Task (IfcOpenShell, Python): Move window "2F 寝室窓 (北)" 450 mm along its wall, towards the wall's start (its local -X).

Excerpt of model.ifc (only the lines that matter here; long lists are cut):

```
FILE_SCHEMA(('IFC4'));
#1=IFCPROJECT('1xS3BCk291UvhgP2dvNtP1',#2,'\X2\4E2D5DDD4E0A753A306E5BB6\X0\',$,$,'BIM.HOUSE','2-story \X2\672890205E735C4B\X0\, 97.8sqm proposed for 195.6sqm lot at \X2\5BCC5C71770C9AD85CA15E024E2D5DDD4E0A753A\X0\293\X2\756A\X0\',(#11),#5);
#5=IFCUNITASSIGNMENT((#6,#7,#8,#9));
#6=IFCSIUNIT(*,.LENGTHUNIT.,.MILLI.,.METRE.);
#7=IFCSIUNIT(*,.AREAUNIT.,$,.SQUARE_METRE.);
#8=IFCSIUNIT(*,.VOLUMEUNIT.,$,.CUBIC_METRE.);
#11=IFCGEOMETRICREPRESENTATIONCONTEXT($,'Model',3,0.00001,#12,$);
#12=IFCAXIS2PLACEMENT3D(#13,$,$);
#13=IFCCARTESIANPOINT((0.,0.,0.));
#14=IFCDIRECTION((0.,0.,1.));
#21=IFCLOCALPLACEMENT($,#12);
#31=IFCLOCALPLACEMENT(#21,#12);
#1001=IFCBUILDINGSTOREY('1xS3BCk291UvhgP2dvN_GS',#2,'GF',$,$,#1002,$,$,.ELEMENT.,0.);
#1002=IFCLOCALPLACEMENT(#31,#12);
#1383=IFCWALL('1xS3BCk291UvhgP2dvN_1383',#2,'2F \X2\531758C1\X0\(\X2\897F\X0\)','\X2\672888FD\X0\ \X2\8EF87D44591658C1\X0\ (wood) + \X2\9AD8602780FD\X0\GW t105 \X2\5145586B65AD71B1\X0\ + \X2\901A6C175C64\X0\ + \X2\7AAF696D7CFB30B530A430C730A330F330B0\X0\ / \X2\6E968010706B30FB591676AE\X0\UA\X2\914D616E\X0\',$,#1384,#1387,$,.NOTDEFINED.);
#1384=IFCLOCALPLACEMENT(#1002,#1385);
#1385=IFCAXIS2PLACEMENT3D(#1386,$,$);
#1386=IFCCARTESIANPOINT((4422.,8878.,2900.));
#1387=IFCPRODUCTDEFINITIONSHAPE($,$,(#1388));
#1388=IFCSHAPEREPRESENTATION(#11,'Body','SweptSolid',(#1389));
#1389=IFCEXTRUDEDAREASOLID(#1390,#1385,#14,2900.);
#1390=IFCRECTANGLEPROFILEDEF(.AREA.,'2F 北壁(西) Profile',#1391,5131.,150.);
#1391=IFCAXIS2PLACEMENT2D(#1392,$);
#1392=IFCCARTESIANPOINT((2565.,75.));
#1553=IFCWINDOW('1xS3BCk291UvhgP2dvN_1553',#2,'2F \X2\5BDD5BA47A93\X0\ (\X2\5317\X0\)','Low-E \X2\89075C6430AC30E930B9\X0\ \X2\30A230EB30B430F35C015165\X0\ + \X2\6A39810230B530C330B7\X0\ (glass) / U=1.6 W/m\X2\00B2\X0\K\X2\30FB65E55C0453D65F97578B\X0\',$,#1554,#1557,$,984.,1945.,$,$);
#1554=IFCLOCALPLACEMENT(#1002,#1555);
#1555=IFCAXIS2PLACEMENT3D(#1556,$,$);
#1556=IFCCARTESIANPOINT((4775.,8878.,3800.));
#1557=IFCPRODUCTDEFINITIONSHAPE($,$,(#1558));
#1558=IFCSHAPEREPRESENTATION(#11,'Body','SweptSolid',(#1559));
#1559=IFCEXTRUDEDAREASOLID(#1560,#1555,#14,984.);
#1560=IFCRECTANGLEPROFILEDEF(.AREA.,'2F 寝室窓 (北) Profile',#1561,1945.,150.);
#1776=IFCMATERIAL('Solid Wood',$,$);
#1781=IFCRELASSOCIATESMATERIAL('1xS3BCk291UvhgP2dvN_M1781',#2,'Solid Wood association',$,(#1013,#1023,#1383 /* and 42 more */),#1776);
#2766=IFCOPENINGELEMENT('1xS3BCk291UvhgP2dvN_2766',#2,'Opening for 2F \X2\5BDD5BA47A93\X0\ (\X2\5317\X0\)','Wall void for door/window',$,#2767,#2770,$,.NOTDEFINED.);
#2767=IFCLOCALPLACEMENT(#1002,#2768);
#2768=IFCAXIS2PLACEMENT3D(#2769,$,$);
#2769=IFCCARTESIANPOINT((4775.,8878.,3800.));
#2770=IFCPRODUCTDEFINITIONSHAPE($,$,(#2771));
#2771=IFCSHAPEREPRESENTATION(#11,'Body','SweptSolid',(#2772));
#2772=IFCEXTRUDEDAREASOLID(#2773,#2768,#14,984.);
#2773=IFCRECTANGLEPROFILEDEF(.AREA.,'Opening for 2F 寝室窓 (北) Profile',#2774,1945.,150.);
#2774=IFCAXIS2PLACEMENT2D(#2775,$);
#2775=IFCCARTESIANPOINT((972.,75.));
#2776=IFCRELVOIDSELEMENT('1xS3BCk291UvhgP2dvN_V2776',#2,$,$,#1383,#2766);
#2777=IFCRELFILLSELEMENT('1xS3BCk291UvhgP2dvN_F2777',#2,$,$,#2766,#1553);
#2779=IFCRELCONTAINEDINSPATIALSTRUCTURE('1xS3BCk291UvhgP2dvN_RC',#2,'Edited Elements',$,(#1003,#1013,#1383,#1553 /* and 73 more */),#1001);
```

```python
import ifcopenshell
import ifcopenshell.api.geometry
import ifcopenshell.util.placement
import ifcopenshell.util.unit

model = ifcopenshell.open("model.ifc")
unit_scale = ifcopenshell.util.unit.calculate_unit_scale(model)

window = model.by_id(1553)
opening = window.FillsVoids[0].RelatingOpeningElement
wall = opening.VoidsElements[0].RelatingBuildingElement

wall_matrix = ifcopenshell.util.placement.get_local_placement(wall.ObjectPlacement)
shift = wall_matrix[:3, 0] * -0.45 / unit_scale
before = ifcopenshell.util.placement.get_local_placement(window.ObjectPlacement)[:3, 3].copy()

# The window is not placed relative to its opening, so move both.
for product in (opening, window):
    matrix = ifcopenshell.util.placement.get_local_placement(product.ObjectPlacement)
    matrix[:3, 3] += shift
    ifcopenshell.api.geometry.edit_object_placement(model, product=product, matrix=matrix, is_si=False)

after = ifcopenshell.util.placement.get_local_placement(window.ObjectPlacement)[:3, 3]
print("window moved by", (after - before).round(3) + 0.0)

model.write("model_v2.ifc")
```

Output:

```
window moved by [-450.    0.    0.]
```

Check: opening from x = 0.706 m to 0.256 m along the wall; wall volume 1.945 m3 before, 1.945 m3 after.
